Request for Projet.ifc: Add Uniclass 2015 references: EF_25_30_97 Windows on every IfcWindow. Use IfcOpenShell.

First a look at what the model holds.

```python
import ifcopenshell

model = ifcopenshell.open("Projet.ifc")
print(model.schema)
print("classifications:", [c.Name for c in model.by_type("IfcClassification")])
for ifc_class in ("IfcDoor", "IfcRoof", "IfcStair", "IfcWall", "IfcWindow"):
    print(ifc_class, len(model.by_type(ifc_class)))
```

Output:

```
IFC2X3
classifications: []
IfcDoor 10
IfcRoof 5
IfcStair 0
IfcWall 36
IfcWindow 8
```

```python
import ifcopenshell
import ifcopenshell.api.classification

model = ifcopenshell.open("Projet.ifc")

# IFC2X3 requires Source and Edition and has no link from the project to the system.
system = model.create_entity("IfcClassification", Source="NBS", Edition="2015", Name="Uniclass 2015")

codes = {
    "IfcWindow": ("EF_25_30_97", "Windows"),
}
for ifc_class, (code, name) in codes.items():
    products = model.by_type(ifc_class)
    ifcopenshell.api.classification.add_reference(
        model, products=products, classification=system, identification=code, name=name
    )
    print(code, len(products))

model.write("Projet_edited.ifc")
```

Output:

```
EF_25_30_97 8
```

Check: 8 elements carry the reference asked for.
